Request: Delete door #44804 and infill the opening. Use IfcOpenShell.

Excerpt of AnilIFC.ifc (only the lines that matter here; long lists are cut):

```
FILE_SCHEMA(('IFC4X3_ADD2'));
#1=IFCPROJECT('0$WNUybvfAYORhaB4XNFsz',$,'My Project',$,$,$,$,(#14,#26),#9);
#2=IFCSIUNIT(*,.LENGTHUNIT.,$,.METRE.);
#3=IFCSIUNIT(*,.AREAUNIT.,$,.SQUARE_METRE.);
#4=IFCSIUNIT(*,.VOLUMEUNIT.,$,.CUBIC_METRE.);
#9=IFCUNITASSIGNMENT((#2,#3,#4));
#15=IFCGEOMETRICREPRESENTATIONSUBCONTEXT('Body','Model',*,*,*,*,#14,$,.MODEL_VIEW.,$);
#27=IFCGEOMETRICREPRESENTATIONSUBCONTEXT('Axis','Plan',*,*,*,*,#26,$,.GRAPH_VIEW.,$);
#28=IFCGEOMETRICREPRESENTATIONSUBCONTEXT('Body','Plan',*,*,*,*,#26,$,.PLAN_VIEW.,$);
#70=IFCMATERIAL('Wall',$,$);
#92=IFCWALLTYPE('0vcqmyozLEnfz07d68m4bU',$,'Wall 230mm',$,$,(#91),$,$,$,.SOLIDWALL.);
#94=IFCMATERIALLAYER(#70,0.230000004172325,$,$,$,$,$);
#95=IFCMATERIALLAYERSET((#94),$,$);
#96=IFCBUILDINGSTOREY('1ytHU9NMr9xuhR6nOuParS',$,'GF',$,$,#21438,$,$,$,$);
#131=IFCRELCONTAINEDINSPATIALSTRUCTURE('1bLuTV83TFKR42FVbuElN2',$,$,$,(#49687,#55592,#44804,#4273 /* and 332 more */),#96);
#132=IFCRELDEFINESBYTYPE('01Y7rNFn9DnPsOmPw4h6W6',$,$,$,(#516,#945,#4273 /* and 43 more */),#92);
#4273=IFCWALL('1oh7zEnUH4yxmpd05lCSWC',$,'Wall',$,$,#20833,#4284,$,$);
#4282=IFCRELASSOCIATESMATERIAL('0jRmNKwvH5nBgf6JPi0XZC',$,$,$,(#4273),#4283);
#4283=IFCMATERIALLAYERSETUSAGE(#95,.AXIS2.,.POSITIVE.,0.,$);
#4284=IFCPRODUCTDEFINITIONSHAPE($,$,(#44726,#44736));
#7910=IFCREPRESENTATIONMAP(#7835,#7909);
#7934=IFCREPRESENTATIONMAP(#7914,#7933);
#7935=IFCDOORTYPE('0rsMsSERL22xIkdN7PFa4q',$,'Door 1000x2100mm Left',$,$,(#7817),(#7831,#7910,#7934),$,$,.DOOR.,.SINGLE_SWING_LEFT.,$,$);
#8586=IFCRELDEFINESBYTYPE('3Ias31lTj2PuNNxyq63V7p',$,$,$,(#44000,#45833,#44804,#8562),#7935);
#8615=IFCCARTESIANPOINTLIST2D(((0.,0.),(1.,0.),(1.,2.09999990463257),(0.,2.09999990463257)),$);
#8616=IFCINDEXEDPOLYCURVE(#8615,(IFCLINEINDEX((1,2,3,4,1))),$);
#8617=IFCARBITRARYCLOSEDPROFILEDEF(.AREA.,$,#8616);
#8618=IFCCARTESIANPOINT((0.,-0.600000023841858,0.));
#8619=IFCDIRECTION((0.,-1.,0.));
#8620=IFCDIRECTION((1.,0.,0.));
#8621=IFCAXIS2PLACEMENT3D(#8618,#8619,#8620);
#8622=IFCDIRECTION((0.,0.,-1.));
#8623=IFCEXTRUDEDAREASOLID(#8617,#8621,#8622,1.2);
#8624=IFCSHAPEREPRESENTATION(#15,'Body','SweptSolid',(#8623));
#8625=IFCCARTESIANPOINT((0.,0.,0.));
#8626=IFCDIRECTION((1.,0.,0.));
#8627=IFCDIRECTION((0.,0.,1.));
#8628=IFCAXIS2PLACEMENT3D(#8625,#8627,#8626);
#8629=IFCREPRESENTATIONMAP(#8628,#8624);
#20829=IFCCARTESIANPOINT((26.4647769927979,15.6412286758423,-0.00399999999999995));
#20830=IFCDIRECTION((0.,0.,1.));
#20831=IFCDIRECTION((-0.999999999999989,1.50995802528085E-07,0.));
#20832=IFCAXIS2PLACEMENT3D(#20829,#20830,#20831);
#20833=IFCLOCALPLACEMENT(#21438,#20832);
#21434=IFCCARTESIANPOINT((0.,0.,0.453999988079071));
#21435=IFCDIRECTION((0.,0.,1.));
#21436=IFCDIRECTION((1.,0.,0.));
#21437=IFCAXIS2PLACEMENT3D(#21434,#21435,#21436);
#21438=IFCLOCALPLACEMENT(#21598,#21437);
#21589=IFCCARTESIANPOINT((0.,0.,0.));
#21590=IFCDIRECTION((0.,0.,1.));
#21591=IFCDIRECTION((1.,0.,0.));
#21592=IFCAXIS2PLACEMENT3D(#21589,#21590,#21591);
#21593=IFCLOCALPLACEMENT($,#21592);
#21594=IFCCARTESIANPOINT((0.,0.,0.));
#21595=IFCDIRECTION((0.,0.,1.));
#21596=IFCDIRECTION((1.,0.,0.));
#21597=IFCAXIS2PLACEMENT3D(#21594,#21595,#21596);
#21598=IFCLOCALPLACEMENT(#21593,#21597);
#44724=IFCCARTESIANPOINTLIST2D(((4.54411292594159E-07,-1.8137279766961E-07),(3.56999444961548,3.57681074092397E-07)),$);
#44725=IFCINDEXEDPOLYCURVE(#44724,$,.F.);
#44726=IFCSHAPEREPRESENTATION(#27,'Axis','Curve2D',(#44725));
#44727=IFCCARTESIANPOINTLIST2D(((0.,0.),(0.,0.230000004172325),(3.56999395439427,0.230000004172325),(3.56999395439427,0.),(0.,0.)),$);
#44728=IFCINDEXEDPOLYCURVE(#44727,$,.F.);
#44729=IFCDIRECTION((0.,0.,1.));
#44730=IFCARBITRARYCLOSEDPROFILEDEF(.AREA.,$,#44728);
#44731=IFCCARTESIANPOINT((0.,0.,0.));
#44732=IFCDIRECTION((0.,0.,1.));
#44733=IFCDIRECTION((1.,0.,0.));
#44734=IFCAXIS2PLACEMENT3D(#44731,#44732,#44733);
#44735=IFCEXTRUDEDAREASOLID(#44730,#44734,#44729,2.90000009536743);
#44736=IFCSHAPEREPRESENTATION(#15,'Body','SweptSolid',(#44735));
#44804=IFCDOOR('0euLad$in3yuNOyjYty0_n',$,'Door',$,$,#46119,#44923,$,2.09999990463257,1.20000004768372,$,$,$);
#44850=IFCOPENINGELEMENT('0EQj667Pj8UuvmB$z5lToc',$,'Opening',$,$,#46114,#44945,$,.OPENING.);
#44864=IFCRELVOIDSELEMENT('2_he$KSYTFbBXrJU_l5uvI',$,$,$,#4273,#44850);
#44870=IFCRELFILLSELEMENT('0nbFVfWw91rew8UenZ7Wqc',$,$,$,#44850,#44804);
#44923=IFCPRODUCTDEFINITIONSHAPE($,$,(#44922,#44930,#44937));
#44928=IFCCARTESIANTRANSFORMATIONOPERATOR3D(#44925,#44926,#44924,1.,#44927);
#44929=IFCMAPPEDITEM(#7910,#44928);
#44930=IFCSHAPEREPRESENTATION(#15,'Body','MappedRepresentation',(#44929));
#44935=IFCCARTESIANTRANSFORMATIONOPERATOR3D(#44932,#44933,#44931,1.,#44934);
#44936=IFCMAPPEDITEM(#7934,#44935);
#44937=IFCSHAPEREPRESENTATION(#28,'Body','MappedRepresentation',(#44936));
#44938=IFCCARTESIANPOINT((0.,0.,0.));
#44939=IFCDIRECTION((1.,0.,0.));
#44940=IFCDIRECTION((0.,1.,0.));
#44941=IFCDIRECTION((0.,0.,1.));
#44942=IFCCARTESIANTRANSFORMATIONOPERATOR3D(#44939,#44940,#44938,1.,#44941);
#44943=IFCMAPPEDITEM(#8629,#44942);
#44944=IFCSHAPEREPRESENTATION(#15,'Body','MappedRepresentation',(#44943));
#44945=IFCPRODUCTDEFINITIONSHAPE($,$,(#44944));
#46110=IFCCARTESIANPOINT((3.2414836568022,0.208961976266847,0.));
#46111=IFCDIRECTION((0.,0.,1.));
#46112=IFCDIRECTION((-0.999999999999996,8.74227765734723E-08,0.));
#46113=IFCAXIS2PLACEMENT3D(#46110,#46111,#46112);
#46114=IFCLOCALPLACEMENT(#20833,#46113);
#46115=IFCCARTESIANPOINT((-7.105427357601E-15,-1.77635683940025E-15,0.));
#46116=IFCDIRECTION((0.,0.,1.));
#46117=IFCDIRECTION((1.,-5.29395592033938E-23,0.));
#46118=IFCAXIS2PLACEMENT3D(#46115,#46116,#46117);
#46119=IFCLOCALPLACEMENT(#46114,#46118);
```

```python
import ifcopenshell
import ifcopenshell.api.feature
import ifcopenshell.api.root
import ifcopenshell.geom
import ifcopenshell.util.shape

model = ifcopenshell.open("AnilIFC.ifc")
settings = ifcopenshell.geom.settings()


def volume(element):
    """Net volume in cubic metres, openings subtracted."""
    shape = ifcopenshell.geom.create_shape(settings, element)
    return ifcopenshell.util.shape.get_volume(shape.geometry)


door = model.by_guid("0euLad$in3yuNOyjYty0_n")
opening = door.FillsVoids[0].RelatingOpeningElement
wall = opening.VoidsElements[0].RelatingBuildingElement
before = volume(wall)

ifcopenshell.api.root.remove_product(model, product=door)
ifcopenshell.api.feature.remove_feature(model, feature=opening)

after = volume(wall)

print(f"wall volume {before:.3f} -> {after:.3f} m3")

model.write("AnilIFC_v2.ifc")
```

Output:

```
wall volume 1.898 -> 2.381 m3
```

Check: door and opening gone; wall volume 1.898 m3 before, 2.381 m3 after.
